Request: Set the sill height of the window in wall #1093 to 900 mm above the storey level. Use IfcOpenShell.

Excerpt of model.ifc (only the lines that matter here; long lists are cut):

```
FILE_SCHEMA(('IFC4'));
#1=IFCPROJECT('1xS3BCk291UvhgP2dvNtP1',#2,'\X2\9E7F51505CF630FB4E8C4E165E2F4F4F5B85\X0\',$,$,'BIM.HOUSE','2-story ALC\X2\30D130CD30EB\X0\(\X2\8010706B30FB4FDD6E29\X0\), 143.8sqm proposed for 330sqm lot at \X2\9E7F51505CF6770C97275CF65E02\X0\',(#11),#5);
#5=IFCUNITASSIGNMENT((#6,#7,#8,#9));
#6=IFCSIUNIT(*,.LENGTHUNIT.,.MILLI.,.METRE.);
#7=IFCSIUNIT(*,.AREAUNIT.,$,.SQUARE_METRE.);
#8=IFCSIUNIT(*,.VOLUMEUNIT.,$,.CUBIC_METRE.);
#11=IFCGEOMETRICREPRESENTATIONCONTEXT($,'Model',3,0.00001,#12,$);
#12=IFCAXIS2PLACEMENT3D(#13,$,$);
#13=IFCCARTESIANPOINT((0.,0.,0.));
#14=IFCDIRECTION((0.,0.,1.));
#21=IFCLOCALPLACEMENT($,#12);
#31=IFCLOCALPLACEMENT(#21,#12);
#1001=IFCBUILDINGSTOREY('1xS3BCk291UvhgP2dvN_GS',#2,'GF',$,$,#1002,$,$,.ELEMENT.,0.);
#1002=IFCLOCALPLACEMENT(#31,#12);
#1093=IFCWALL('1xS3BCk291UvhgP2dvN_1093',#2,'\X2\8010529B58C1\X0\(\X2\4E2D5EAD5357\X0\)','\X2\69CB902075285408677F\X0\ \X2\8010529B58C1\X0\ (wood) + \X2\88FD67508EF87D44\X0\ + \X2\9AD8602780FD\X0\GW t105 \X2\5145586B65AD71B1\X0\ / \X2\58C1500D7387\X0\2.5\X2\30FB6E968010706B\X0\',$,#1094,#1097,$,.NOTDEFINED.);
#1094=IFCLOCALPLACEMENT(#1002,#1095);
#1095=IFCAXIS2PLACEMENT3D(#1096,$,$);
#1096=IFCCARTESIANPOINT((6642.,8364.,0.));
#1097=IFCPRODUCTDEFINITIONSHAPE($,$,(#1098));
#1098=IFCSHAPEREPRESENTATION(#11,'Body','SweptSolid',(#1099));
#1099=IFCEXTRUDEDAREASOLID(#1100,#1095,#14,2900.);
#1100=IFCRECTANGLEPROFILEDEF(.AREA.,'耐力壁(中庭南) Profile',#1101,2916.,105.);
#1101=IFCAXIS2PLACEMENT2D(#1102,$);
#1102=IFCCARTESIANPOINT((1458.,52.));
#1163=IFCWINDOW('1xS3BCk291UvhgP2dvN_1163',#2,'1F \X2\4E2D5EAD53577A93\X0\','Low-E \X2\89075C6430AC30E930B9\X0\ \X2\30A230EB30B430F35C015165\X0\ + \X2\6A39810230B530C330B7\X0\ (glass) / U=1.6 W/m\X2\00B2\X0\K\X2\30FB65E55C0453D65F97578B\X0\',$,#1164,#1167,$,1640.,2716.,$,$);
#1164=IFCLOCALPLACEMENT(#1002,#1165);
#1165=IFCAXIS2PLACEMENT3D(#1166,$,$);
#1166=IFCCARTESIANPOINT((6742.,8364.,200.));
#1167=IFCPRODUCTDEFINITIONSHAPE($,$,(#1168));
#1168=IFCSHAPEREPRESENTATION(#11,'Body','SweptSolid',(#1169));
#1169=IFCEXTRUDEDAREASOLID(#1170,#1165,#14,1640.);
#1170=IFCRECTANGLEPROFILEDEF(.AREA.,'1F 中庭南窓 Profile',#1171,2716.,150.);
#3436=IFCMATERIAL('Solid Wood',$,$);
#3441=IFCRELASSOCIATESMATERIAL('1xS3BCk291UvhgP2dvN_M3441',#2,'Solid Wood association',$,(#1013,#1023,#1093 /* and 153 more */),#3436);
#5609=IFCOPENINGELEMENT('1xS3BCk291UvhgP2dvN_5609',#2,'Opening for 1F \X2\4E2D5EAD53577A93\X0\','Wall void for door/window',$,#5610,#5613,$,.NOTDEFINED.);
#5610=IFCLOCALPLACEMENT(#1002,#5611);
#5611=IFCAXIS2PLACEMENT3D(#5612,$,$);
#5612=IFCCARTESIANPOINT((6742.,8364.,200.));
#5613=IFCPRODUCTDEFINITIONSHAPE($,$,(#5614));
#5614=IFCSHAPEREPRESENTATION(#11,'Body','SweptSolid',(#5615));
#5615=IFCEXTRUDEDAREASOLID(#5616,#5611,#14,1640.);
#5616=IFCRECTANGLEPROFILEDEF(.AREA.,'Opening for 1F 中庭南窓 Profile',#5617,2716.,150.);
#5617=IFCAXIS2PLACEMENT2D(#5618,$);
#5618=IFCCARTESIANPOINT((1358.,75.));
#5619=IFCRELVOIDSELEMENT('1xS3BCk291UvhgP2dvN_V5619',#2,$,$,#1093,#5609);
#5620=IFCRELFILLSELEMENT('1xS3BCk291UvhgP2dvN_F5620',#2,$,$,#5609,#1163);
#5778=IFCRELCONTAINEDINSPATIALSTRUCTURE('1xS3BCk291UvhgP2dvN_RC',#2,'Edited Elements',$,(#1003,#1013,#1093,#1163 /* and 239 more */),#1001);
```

```python
import numpy as np
import ifcopenshell
import ifcopenshell.api.geometry
import ifcopenshell.geom
import ifcopenshell.util.element
import ifcopenshell.util.placement
import ifcopenshell.util.shape
import ifcopenshell.util.unit

model = ifcopenshell.open("model.ifc")
unit_scale = ifcopenshell.util.unit.calculate_unit_scale(model)

window = model.by_guid("1xS3BCk291UvhgP2dvN_1163")
opening = window.FillsVoids[0].RelatingOpeningElement
storey = ifcopenshell.util.element.get_container(window, ifc_class="IfcBuildingStorey")
level = ifcopenshell.util.placement.get_local_placement(storey.ObjectPlacement)[2, 3]

# The opening's origin need not be at the sill, so measure its lowest point.
shape = ifcopenshell.geom.create_shape(ifcopenshell.geom.settings(), opening)
bottom = ifcopenshell.util.shape.get_shape_bottom_elevation(shape, shape.geometry) / unit_scale
dz = level + 900.0 - bottom

shift = np.array([0.0, 0.0, dz])
# The window is not placed relative to its opening, so move both.
for product in (opening, window):
    matrix = ifcopenshell.util.placement.get_local_placement(product.ObjectPlacement)
    matrix[:3, 3] += shift
    ifcopenshell.api.geometry.edit_object_placement(model, product=product, matrix=matrix, is_si=False)

print(f"moved by {dz * unit_scale:+.3f} m")

model.write("model-out.ifc")
```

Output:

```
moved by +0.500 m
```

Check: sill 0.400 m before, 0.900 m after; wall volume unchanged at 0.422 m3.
